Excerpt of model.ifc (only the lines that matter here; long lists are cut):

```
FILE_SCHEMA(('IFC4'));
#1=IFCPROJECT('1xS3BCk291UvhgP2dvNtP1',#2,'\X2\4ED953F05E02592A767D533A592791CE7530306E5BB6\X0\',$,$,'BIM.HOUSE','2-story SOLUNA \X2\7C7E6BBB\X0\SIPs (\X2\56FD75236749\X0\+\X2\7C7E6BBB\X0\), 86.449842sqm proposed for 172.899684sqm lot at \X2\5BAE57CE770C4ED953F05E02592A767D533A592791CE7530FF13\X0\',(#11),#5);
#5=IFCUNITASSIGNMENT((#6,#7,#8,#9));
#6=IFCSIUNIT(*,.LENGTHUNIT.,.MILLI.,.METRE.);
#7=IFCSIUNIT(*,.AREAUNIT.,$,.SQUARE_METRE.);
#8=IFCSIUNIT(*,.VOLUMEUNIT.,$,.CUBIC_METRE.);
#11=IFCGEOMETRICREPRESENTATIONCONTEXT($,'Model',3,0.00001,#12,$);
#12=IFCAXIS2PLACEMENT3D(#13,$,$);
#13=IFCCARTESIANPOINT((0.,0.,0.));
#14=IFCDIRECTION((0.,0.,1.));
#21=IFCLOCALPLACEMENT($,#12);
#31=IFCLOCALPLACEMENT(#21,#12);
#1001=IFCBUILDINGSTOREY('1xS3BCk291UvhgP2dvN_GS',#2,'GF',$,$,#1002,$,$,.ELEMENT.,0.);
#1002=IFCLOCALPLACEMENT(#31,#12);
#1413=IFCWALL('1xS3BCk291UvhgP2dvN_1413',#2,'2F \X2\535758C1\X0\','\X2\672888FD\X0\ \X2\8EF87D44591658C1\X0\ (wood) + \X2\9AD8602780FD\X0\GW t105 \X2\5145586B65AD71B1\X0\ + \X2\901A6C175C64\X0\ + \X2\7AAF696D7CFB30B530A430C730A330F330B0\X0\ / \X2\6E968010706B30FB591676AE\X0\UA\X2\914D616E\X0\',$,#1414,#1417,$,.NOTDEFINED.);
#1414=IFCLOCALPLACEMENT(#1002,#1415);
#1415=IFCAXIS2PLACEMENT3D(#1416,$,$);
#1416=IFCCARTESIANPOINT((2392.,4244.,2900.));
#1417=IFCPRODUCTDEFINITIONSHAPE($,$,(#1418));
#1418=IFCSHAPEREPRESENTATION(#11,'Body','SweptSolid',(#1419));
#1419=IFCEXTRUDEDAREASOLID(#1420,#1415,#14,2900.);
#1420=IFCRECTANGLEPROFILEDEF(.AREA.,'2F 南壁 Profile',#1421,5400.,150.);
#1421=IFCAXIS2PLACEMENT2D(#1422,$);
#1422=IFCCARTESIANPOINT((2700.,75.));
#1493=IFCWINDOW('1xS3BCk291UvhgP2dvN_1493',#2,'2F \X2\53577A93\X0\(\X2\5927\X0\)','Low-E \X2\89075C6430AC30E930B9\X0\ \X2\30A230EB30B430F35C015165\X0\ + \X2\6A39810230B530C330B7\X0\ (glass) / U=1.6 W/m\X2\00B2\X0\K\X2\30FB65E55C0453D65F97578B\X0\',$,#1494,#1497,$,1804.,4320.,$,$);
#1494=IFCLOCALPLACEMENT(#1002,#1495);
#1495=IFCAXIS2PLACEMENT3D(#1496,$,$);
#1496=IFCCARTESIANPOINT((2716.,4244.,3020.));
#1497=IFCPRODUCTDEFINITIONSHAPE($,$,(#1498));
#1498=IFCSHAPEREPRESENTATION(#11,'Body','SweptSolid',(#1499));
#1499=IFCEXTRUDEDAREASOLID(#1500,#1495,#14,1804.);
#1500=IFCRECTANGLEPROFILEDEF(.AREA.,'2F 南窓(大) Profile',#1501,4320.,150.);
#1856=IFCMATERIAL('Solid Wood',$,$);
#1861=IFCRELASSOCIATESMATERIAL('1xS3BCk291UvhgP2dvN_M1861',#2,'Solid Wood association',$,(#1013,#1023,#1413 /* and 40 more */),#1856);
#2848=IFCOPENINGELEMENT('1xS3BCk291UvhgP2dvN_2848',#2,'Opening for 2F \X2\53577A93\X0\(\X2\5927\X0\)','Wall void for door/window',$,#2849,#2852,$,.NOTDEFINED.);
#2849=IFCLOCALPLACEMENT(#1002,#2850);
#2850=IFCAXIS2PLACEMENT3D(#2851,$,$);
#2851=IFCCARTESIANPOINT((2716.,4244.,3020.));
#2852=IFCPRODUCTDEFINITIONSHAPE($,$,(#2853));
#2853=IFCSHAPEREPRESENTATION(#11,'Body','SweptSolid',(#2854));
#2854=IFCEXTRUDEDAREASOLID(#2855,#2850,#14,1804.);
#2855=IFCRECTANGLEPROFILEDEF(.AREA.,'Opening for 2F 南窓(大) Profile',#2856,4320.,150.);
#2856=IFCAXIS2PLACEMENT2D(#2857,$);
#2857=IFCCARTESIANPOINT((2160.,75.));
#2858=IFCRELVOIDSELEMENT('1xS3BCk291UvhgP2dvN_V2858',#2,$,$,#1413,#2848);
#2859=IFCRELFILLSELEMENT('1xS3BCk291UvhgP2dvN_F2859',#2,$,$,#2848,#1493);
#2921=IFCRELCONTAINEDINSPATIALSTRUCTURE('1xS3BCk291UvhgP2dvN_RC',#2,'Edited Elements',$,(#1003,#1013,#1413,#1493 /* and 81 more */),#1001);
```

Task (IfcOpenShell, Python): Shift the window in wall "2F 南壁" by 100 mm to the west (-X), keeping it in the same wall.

```python
import ifcopenshell
import ifcopenshell.api.geometry
import ifcopenshell.util.placement
import ifcopenshell.util.unit

model = ifcopenshell.open("model.ifc")
unit_scale = ifcopenshell.util.unit.calculate_unit_scale(model)

window = model.by_id(1493)
opening = window.FillsVoids[0].RelatingOpeningElement
wall = opening.VoidsElements[0].RelatingBuildingElement

wall_matrix = ifcopenshell.util.placement.get_local_placement(wall.ObjectPlacement)
shift = wall_matrix[:3, 0] * -0.1 / unit_scale
before = ifcopenshell.util.placement.get_local_placement(window.ObjectPlacement)[:3, 3].copy()

# The window is not placed relative to its opening, so move both.
for product in (opening, window):
    matrix = ifcopenshell.util.placement.get_local_placement(product.ObjectPlacement)
    matrix[:3, 3] += shift
    ifcopenshell.api.geometry.edit_object_placement(model, product=product, matrix=matrix, is_si=False)

after = ifcopenshell.util.placement.get_local_placement(window.ObjectPlacement)[:3, 3]
print("window moved by", (after - before).round(3) + 0.0)

model.write("model_edited.ifc")
```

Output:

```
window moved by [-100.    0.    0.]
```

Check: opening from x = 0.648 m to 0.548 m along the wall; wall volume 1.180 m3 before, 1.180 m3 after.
